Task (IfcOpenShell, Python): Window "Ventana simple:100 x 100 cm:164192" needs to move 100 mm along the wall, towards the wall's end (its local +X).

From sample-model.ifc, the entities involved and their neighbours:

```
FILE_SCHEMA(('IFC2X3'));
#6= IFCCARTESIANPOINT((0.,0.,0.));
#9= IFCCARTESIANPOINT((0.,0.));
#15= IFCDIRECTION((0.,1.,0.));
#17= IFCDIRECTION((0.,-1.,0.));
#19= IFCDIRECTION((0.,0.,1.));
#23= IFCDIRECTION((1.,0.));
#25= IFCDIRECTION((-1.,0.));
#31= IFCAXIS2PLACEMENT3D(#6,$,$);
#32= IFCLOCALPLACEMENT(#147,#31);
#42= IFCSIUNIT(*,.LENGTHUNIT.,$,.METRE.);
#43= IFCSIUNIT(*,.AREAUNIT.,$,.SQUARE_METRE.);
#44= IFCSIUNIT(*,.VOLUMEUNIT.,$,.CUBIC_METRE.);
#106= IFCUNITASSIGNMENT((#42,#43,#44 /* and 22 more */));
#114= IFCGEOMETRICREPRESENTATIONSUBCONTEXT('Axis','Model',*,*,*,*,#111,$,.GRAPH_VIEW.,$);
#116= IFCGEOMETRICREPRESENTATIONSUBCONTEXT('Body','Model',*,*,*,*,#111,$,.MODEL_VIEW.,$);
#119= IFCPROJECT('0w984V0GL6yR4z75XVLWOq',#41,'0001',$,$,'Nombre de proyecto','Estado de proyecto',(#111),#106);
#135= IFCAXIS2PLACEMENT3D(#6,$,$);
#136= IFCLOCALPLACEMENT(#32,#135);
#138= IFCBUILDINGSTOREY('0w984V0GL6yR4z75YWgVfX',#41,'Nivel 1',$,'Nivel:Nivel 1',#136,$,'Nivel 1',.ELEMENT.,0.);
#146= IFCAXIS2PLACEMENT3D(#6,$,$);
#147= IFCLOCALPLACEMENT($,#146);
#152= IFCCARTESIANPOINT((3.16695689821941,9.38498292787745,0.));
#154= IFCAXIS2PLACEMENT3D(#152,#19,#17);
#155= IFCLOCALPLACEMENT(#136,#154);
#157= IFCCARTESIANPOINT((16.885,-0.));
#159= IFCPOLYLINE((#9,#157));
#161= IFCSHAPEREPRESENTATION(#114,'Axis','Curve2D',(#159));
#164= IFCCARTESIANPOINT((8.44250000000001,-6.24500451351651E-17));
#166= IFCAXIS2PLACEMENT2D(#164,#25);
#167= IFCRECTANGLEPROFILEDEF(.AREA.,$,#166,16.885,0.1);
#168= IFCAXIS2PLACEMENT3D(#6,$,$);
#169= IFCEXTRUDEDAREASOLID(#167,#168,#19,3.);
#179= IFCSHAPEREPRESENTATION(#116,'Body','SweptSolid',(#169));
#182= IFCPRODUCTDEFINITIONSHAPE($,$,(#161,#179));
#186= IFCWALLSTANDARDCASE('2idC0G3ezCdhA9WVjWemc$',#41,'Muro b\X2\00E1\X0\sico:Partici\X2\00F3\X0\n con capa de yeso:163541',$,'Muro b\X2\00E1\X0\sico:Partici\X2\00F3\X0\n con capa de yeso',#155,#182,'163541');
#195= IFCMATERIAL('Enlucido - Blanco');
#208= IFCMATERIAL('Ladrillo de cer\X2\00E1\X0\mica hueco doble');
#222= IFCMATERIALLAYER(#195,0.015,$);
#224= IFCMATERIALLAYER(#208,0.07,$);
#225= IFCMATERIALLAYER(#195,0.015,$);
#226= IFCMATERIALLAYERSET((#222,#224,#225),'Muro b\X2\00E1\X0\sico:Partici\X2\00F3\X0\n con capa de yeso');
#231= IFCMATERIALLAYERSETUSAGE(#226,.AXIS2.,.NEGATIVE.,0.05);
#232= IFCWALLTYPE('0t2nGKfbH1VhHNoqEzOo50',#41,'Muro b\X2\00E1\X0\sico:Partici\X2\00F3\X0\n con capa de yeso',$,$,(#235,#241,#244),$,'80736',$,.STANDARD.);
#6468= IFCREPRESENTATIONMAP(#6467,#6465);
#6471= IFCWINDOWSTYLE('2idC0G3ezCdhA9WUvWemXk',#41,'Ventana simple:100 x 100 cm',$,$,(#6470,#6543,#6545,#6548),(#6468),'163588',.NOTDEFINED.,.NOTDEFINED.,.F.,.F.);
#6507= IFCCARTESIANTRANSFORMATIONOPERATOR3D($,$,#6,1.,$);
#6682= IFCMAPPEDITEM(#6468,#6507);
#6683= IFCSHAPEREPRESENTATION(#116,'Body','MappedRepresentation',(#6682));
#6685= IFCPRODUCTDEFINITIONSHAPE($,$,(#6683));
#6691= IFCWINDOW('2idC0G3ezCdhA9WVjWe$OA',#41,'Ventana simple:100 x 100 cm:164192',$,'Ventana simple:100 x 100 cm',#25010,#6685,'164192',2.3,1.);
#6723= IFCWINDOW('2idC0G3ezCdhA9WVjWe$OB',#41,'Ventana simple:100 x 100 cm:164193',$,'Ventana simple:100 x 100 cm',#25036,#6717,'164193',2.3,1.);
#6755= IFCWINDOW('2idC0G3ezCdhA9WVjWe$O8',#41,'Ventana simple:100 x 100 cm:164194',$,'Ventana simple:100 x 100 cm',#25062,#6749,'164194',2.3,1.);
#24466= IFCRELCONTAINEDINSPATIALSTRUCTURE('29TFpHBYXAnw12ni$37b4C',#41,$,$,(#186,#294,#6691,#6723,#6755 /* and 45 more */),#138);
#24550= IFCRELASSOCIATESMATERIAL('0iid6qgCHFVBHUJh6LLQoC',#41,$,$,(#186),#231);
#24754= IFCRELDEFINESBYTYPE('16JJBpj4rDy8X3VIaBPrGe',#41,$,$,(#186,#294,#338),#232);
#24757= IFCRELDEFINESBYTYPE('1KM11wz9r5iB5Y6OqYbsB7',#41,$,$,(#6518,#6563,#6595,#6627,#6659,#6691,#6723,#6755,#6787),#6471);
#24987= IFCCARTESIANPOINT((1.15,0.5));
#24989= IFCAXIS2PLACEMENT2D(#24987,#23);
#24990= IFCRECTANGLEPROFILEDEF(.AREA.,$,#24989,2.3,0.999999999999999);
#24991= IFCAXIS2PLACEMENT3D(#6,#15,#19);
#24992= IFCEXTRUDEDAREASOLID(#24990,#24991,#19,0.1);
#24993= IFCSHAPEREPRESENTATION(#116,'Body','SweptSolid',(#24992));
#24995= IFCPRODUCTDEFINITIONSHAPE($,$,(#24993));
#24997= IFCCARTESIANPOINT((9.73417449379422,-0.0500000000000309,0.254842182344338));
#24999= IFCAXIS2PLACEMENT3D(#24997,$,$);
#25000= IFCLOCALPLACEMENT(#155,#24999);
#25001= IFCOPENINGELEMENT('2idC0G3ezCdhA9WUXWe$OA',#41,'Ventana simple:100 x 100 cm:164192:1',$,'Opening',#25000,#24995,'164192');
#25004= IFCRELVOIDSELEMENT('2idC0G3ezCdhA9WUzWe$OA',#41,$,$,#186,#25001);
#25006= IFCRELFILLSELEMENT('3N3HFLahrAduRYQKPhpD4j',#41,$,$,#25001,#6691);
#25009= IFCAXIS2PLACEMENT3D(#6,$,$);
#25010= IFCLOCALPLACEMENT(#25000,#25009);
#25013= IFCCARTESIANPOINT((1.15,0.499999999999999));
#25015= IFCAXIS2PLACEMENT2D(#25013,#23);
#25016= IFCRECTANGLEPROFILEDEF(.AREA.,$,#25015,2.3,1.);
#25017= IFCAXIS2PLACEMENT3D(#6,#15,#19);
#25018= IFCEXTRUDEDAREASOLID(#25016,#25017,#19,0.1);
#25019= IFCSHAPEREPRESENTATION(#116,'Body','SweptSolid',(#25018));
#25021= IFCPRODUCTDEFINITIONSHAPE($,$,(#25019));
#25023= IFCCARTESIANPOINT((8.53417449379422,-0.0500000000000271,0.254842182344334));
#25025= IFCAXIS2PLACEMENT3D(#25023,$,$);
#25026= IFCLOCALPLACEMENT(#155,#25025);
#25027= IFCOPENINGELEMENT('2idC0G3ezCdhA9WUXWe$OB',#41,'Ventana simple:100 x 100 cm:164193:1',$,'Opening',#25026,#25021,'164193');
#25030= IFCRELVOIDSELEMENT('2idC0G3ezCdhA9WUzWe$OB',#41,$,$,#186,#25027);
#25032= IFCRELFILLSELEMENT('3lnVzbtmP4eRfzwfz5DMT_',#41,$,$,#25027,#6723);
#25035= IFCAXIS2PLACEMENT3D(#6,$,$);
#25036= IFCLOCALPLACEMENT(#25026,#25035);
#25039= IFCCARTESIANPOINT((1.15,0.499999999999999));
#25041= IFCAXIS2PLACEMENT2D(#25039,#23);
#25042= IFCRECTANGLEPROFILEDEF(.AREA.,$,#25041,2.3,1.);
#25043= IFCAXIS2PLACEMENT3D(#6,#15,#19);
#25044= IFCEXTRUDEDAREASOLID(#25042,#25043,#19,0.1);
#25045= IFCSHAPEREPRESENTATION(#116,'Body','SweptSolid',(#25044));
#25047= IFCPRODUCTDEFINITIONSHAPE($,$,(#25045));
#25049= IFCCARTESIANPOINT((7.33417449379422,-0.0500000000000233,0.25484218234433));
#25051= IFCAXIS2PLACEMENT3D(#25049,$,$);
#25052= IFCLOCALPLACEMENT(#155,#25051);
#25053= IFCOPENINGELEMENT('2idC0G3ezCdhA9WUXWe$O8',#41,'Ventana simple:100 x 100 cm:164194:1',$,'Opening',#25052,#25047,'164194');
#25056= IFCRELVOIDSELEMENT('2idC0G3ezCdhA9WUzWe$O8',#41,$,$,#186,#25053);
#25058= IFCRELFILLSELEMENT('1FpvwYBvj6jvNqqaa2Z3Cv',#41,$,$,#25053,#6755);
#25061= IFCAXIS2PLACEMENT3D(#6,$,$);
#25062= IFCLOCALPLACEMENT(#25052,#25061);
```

```python
import ifcopenshell
import ifcopenshell.api.geometry
import ifcopenshell.util.placement

model = ifcopenshell.open("sample-model.ifc")

window = model.by_id(6691)
opening = window.FillsVoids[0].RelatingOpeningElement
wall = opening.VoidsElements[0].RelatingBuildingElement

wall_matrix = ifcopenshell.util.placement.get_local_placement(wall.ObjectPlacement)
shift = wall_matrix[:3, 0] * 0.1
before = ifcopenshell.util.placement.get_local_placement(window.ObjectPlacement)[:3, 3].copy()

# The window is placed relative to its opening, so it follows when the opening moves.
matrix = ifcopenshell.util.placement.get_local_placement(opening.ObjectPlacement)
matrix[:3, 3] += shift
ifcopenshell.api.geometry.edit_object_placement(
    model, product=opening, matrix=matrix, is_si=False, should_transform_children=True
)

after = ifcopenshell.util.placement.get_local_placement(window.ObjectPlacement)[:3, 3]
print("window moved by", (after - before).round(3) + 0.0)

model.write("sample-model_updated.ifc")
```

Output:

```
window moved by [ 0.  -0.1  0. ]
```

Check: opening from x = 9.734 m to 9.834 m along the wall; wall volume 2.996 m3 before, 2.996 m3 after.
